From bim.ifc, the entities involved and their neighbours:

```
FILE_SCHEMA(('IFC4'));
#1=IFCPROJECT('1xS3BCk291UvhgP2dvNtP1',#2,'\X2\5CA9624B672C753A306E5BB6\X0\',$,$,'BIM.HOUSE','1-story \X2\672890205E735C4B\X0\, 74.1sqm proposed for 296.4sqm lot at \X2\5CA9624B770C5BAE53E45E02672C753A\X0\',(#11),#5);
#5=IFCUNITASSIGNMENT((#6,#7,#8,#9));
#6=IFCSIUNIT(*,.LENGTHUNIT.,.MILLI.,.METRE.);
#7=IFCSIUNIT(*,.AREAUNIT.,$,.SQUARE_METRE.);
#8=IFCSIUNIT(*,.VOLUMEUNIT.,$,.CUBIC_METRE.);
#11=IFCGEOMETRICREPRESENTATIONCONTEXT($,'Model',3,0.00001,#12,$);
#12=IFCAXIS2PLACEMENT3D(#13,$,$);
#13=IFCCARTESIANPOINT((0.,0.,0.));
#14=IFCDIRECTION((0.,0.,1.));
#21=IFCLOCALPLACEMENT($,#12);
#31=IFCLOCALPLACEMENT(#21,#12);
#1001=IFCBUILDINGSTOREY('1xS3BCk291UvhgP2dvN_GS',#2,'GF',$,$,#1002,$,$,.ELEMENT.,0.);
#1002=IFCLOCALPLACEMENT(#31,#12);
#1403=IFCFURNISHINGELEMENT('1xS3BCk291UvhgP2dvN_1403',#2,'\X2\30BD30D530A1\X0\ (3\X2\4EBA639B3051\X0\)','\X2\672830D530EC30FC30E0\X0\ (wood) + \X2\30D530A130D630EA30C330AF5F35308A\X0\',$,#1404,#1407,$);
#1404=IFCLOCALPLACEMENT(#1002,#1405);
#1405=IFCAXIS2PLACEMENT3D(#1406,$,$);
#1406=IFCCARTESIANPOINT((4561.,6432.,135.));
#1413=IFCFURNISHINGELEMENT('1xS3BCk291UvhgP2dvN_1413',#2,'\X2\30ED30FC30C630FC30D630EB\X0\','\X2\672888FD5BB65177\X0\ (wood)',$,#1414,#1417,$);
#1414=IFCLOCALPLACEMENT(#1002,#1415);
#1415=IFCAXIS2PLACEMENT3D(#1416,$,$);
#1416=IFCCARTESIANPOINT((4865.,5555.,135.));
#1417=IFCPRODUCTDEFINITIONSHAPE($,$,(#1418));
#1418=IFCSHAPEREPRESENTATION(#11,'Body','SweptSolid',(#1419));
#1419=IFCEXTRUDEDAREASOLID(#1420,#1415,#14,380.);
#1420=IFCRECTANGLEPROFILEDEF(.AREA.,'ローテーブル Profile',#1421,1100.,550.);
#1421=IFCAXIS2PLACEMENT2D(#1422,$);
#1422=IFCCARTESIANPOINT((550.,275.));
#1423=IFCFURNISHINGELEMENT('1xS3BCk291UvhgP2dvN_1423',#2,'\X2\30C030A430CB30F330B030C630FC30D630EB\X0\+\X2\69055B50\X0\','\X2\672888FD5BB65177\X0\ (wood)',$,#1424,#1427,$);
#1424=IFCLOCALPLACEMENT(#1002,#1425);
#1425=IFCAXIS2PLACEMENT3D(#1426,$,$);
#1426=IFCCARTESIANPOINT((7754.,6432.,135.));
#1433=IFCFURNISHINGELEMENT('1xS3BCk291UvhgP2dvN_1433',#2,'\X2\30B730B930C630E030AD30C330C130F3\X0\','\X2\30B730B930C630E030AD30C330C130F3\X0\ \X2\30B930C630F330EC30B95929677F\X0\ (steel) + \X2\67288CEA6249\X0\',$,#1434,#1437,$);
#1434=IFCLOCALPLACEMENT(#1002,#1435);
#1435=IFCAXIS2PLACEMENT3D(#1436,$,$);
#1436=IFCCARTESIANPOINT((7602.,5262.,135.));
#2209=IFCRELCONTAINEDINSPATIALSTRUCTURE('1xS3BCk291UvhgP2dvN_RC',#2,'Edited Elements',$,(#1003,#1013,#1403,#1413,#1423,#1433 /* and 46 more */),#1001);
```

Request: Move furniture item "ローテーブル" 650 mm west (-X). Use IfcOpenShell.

```python
import ifcopenshell
import ifcopenshell.api.geometry
import ifcopenshell.util.placement
import ifcopenshell.util.unit

model = ifcopenshell.open("bim.ifc")
unit_scale = ifcopenshell.util.unit.calculate_unit_scale(model)

item = model.by_guid("1xS3BCk291UvhgP2dvN_1413")
matrix = ifcopenshell.util.placement.get_local_placement(item.ObjectPlacement)
matrix[0, 3] -= 0.65 / unit_scale
ifcopenshell.api.geometry.edit_object_placement(model, product=item, matrix=matrix, is_si=False)

print(ifcopenshell.util.placement.get_local_placement(item.ObjectPlacement).round(3) + 0.0)

model.write("bim_edited.ifc")
```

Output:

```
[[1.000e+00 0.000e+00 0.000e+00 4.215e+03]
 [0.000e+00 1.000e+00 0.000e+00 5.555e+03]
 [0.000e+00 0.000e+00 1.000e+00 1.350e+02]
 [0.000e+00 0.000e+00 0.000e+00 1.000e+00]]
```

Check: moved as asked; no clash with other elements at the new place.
